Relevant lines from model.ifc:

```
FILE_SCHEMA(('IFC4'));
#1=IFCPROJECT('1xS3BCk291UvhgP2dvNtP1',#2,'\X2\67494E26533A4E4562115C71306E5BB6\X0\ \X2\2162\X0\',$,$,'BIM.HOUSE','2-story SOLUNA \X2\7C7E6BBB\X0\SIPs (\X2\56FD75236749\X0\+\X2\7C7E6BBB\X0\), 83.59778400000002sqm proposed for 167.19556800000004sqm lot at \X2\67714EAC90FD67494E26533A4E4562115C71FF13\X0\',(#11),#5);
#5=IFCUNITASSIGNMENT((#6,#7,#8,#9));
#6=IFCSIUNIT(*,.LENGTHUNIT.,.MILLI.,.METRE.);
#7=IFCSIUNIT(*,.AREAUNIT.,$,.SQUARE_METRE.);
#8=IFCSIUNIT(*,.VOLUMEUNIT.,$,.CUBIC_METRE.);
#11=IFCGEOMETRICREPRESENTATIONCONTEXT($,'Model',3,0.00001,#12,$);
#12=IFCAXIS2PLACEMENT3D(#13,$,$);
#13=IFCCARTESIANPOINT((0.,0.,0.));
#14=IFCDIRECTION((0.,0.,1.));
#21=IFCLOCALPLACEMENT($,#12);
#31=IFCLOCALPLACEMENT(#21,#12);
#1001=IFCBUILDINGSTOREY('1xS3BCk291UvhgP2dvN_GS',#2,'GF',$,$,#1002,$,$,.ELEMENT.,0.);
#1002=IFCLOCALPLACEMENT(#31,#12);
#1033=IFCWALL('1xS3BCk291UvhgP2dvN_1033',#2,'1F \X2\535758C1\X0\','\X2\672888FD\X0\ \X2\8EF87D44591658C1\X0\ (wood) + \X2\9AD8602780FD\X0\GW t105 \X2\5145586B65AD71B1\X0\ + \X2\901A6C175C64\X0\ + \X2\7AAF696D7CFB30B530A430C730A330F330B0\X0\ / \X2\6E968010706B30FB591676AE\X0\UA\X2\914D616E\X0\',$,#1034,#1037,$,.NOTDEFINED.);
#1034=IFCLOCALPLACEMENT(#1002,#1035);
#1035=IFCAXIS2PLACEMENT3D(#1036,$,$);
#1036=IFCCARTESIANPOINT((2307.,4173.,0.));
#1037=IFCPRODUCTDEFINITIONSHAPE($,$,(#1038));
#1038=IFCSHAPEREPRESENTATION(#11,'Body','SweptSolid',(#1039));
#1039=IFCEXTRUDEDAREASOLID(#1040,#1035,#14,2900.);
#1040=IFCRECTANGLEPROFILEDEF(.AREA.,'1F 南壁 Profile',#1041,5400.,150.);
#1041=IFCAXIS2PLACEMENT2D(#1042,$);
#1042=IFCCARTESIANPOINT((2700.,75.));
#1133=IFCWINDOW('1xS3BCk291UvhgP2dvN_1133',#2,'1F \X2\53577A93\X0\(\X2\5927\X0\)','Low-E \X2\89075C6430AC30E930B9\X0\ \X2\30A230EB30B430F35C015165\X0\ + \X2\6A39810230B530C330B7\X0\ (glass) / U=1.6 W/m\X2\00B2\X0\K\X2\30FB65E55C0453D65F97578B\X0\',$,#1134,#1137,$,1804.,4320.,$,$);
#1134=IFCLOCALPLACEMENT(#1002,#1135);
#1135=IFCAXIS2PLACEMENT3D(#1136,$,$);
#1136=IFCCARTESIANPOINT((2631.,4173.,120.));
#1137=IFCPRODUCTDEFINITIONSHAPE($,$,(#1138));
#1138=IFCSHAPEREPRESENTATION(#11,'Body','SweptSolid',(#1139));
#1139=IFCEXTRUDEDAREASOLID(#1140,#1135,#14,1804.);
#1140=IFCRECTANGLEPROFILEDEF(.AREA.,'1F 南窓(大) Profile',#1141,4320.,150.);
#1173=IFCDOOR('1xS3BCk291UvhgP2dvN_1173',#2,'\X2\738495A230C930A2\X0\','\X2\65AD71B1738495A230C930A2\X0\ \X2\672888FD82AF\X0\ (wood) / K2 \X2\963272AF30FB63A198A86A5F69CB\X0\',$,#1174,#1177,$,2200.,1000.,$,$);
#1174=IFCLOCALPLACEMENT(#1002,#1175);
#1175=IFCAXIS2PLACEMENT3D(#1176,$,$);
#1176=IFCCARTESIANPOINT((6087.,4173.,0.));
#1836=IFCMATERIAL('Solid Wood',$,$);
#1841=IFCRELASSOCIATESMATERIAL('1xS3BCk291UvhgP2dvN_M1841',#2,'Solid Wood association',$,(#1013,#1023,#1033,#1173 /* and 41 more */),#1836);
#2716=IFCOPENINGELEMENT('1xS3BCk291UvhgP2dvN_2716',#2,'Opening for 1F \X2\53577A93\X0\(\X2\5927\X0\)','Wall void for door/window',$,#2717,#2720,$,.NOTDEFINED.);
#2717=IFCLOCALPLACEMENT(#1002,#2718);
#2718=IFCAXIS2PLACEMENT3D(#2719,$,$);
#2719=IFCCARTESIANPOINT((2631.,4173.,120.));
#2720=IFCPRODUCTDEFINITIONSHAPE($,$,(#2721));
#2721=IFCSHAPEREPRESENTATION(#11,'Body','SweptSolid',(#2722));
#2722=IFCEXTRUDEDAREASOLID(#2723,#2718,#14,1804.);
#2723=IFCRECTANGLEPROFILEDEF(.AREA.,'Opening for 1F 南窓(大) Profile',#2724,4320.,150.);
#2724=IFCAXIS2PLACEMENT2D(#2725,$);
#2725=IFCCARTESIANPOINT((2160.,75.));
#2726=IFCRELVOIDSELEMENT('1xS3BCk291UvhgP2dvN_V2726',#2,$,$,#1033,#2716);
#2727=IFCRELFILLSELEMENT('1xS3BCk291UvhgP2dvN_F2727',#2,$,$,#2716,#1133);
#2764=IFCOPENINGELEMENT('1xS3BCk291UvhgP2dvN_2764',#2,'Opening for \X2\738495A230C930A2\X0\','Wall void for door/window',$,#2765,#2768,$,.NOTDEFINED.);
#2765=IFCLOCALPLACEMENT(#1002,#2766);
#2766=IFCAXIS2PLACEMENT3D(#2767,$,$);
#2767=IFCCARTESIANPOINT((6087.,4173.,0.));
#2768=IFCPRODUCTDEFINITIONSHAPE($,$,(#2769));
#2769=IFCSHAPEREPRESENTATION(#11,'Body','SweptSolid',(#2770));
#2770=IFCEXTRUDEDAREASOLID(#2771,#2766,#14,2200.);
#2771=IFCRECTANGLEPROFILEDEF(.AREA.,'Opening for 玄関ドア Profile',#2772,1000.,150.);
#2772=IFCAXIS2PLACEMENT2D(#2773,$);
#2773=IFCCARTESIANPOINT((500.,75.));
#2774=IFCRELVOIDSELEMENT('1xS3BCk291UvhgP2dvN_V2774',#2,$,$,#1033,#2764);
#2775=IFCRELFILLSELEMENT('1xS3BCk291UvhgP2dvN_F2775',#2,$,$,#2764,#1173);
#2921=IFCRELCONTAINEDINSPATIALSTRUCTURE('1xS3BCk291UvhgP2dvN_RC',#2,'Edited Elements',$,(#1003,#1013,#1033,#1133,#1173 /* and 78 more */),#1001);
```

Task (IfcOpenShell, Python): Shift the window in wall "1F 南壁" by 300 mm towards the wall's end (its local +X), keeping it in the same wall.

```python
import ifcopenshell
import ifcopenshell.api.geometry
import ifcopenshell.util.placement

model = ifcopenshell.open("model.ifc")

window = model.by_guid("1xS3BCk291UvhgP2dvN_1133")
opening = window.FillsVoids[0].RelatingOpeningElement
wall = opening.VoidsElements[0].RelatingBuildingElement

wall_matrix = ifcopenshell.util.placement.get_local_placement(wall.ObjectPlacement)
shift = wall_matrix[:3, 0] * 300.0
before = ifcopenshell.util.placement.get_local_placement(window.ObjectPlacement)[:3, 3].copy()

# The window is not placed relative to its opening, so move both.
for product in (opening, window):
    matrix = ifcopenshell.util.placement.get_local_placement(product.ObjectPlacement)
    matrix[:3, 3] += shift
    ifcopenshell.api.geometry.edit_object_placement(model, product=product, matrix=matrix, is_si=False)

after = ifcopenshell.util.placement.get_local_placement(window.ObjectPlacement)[:3, 3]
print("window moved by", (after - before).round(3) + 0.0)

model.write("model_v2.ifc")
```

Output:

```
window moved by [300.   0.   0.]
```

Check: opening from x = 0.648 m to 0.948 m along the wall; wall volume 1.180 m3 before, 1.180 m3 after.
